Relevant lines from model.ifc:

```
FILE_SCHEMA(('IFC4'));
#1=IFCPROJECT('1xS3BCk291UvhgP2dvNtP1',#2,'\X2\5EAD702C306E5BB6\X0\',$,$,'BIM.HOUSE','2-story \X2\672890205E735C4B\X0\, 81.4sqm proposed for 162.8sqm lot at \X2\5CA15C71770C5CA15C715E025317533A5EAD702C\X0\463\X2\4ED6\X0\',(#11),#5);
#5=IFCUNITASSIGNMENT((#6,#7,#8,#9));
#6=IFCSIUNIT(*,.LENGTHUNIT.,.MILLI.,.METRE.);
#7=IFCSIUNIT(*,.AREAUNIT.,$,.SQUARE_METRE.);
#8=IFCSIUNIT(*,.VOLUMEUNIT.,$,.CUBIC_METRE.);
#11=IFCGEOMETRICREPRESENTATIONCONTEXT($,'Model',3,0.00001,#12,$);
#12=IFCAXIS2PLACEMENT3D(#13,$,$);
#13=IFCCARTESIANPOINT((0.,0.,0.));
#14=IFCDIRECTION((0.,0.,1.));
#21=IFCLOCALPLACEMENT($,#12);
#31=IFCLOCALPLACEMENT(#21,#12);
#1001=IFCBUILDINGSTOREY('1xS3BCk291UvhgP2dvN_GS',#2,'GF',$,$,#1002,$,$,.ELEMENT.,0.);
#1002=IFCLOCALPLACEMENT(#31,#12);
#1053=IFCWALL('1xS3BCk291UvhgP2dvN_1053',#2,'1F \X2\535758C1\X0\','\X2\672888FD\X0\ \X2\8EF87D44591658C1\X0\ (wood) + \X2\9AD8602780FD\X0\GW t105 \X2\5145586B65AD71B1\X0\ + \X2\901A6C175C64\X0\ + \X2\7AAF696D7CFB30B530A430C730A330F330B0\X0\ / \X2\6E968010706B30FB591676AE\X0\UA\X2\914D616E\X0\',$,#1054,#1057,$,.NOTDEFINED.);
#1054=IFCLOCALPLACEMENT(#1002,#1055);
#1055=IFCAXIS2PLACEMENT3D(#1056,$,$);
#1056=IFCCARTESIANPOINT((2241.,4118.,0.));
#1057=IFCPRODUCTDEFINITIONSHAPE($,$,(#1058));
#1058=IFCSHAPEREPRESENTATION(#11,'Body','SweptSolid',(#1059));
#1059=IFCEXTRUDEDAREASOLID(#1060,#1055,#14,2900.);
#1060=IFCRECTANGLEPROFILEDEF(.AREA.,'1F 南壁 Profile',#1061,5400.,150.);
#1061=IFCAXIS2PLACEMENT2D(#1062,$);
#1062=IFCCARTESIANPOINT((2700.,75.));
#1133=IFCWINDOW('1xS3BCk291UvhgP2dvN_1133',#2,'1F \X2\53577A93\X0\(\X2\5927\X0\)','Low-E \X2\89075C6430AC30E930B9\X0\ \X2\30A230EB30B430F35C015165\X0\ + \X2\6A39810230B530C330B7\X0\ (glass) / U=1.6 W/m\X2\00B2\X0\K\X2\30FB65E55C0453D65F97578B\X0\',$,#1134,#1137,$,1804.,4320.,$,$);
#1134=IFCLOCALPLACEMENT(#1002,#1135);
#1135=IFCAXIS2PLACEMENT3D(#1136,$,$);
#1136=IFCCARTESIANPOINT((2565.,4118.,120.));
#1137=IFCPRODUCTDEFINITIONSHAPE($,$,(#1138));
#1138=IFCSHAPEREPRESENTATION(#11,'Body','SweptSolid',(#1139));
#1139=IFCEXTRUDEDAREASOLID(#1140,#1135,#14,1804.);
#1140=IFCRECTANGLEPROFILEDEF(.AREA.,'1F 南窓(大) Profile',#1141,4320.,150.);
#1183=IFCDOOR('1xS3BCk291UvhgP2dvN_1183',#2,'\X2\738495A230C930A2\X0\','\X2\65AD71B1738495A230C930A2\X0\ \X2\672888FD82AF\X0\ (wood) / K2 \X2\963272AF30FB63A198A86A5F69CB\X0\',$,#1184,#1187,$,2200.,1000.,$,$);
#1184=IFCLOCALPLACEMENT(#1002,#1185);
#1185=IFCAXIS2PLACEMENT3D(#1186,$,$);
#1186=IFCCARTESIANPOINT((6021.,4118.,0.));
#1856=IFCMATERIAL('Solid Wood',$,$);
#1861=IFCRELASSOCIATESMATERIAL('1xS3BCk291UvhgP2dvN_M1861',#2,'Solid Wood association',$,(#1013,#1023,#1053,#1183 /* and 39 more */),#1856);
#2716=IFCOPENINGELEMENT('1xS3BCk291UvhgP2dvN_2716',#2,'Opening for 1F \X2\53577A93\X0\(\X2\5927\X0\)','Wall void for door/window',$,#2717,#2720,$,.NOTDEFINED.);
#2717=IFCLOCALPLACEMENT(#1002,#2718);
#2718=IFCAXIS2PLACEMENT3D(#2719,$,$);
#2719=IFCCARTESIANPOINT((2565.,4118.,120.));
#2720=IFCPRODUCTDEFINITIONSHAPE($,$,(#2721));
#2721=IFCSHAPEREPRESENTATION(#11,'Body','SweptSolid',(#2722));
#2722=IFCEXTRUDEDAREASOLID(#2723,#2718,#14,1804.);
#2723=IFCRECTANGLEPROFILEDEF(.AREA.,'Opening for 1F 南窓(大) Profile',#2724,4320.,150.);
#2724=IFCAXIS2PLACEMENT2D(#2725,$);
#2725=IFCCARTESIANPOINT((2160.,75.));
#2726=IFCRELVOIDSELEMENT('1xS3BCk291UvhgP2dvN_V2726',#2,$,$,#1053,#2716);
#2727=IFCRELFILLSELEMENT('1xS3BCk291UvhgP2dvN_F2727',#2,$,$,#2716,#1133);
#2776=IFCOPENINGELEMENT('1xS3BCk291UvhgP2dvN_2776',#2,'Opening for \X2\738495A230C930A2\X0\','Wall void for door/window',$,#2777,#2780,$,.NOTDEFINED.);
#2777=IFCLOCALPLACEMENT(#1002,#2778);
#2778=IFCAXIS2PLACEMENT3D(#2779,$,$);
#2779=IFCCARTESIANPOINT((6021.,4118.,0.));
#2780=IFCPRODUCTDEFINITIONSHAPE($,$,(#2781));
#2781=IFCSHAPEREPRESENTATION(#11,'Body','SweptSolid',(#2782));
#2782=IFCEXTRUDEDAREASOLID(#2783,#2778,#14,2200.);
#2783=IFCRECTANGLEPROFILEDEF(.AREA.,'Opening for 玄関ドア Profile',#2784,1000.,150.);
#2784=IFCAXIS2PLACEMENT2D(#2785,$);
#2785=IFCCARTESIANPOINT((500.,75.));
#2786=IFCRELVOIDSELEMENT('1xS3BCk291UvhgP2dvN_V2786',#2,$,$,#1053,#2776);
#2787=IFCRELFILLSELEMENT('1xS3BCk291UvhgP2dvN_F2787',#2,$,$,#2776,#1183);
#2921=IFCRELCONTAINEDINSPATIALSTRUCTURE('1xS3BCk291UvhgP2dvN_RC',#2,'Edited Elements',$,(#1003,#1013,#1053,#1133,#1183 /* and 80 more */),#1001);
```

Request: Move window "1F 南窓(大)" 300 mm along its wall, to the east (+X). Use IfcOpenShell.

```python
import ifcopenshell
import ifcopenshell.api.geometry
import ifcopenshell.util.placement
import ifcopenshell.util.unit

model = ifcopenshell.open("model.ifc")
unit_scale = ifcopenshell.util.unit.calculate_unit_scale(model)

window = model.by_guid("1xS3BCk291UvhgP2dvN_1133")
opening = window.FillsVoids[0].RelatingOpeningElement
wall = opening.VoidsElements[0].RelatingBuildingElement

wall_matrix = ifcopenshell.util.placement.get_local_placement(wall.ObjectPlacement)
shift = wall_matrix[:3, 0] * 0.3 / unit_scale
before = ifcopenshell.util.placement.get_local_placement(window.ObjectPlacement)[:3, 3].copy()

# The window is not placed relative to its opening, so move both.
for product in (opening, window):
    matrix = ifcopenshell.util.placement.get_local_placement(product.ObjectPlacement)
    matrix[:3, 3] += shift
    ifcopenshell.api.geometry.edit_object_placement(model, product=product, matrix=matrix, is_si=False)

after = ifcopenshell.util.placement.get_local_placement(window.ObjectPlacement)[:3, 3]
print("window moved by", (after - before).round(3) + 0.0)

model.write("model_updated.ifc")
```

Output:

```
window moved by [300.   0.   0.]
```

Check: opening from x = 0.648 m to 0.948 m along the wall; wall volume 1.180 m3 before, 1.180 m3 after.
